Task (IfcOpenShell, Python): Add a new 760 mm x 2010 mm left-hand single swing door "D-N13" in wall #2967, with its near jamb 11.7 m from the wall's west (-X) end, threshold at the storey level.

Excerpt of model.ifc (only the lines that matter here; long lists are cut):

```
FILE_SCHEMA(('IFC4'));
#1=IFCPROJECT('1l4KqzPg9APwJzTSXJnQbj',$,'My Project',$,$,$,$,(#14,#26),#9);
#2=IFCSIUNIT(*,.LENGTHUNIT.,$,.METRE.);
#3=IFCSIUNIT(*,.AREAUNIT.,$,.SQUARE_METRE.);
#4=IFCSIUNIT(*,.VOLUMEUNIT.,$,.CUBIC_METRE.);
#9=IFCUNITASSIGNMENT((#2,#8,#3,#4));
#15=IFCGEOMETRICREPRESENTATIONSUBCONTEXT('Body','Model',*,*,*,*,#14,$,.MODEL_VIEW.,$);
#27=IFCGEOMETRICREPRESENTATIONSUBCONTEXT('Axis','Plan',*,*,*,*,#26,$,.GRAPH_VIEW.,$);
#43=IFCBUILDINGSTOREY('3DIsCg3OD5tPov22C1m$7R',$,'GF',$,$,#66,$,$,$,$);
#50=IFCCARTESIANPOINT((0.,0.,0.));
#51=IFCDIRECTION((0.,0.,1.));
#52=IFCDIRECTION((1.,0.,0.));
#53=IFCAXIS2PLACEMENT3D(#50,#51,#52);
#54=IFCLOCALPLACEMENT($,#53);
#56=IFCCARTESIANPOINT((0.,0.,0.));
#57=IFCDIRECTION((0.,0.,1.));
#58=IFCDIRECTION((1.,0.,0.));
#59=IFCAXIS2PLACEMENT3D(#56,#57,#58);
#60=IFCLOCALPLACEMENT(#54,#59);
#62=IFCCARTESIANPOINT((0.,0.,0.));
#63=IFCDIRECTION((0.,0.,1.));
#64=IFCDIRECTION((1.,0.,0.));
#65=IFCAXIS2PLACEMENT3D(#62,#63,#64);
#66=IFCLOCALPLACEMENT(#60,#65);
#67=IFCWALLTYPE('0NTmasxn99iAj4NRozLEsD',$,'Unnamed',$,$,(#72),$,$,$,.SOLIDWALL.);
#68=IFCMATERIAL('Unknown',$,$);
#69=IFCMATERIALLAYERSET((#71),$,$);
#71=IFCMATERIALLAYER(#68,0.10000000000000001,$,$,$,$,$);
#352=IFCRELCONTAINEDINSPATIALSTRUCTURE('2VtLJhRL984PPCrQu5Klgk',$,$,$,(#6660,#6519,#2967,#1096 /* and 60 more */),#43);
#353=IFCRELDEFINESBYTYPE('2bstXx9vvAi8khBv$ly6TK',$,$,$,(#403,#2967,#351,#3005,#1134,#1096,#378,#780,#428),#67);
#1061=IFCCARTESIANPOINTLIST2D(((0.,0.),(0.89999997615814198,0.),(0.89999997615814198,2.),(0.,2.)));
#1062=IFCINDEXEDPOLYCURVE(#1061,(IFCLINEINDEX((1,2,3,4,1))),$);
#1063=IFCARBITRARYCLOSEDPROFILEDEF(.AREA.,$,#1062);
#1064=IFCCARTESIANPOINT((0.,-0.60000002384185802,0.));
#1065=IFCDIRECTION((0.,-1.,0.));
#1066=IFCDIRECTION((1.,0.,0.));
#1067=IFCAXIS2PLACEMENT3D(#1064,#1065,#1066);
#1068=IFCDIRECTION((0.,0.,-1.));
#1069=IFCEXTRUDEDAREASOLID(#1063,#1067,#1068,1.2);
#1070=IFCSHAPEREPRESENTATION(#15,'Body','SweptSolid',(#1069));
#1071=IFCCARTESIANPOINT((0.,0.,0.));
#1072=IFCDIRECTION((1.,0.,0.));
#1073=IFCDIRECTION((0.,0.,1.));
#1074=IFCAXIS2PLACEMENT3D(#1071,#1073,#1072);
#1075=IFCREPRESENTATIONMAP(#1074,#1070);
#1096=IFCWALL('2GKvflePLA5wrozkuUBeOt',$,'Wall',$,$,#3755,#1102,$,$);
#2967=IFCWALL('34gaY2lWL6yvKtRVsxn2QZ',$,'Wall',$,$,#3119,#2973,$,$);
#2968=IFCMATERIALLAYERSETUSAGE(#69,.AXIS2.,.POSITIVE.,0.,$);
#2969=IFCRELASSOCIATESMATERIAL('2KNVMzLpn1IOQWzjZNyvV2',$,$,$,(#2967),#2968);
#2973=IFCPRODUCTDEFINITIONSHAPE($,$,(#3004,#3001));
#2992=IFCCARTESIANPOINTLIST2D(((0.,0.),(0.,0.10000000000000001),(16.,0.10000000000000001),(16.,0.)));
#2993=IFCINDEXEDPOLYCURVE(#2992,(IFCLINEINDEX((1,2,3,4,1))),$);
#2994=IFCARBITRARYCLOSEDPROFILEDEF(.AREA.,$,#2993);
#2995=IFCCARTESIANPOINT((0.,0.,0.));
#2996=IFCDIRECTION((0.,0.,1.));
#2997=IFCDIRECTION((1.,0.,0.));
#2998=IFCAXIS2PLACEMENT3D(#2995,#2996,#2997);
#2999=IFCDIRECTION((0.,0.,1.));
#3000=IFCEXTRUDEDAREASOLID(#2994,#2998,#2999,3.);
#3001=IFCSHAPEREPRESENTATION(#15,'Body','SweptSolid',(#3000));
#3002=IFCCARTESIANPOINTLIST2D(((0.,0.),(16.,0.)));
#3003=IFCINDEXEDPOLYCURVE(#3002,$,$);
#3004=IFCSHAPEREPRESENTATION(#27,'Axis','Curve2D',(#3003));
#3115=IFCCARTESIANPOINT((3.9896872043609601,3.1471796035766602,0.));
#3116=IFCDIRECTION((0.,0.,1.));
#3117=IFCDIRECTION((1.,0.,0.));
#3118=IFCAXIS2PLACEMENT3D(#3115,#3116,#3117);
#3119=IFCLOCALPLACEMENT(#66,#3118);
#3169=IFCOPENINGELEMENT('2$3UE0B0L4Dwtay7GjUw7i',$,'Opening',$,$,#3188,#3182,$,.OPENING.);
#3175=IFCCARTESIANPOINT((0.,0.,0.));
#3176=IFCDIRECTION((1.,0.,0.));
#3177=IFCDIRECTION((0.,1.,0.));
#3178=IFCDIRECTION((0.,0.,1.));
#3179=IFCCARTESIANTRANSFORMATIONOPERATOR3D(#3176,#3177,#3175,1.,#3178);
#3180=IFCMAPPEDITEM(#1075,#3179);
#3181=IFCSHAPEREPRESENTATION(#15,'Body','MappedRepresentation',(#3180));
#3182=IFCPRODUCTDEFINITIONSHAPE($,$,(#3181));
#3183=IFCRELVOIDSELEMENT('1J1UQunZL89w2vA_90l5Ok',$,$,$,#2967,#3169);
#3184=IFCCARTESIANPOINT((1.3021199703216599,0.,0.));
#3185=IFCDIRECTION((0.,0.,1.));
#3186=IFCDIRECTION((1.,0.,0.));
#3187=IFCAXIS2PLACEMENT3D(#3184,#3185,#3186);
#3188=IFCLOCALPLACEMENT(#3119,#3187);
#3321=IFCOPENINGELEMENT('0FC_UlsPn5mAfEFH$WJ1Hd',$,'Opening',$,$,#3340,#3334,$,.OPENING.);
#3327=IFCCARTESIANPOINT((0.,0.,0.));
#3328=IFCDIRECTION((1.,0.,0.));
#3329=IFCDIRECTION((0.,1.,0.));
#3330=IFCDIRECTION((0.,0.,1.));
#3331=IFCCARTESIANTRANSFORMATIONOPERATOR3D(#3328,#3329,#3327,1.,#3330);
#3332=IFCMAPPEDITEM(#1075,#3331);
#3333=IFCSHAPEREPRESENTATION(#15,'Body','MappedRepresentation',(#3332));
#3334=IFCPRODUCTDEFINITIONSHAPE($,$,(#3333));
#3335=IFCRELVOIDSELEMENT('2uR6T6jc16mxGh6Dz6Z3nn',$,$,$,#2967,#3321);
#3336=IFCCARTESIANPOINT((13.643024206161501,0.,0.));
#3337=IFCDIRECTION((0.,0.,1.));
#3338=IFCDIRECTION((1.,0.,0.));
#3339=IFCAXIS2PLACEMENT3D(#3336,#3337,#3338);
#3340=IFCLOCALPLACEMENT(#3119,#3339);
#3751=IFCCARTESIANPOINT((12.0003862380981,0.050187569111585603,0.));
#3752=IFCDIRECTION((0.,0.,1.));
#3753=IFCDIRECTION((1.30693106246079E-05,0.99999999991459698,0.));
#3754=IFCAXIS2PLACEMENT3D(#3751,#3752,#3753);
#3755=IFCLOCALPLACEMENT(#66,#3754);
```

```python
import numpy as np
import ifcopenshell
import ifcopenshell.api.feature
import ifcopenshell.api.geometry
import ifcopenshell.api.root
import ifcopenshell.api.spatial
import ifcopenshell.geom
import ifcopenshell.util.element
import ifcopenshell.util.placement
import ifcopenshell.util.representation
import ifcopenshell.util.shape
import ifcopenshell.util.unit

model = ifcopenshell.open("model.ifc")
unit_scale = ifcopenshell.util.unit.calculate_unit_scale(model)
settings = ifcopenshell.geom.settings()


def volume(element):
    """Net volume in cubic metres, openings subtracted."""
    shape = ifcopenshell.geom.create_shape(settings, element)
    return ifcopenshell.util.shape.get_volume(shape.geometry)


wall = model.by_id(2967)
storey = ifcopenshell.util.element.get_container(wall, ifc_class="IfcBuildingStorey")
context = ifcopenshell.util.representation.get_context(model, "Model", "Body", "MODEL_VIEW")
before = volume(wall)

width, height, from_end, sill = 0.76, 2.01, 11.7, 0.0  # metres

# The wall runs along its own X axis, and the end named is its -X end.
wall_shape = ifcopenshell.geom.create_shape(settings, wall)
x, y, z = ifcopenshell.util.shape.get_vertices(wall_shape.geometry).T
start = x.min() + from_end
face, thickness = float(y.min()), float(y.max() - y.min())
wall_matrix = ifcopenshell.util.placement.get_local_placement(wall.ObjectPlacement)
level = ifcopenshell.util.placement.get_local_placement(storey.ObjectPlacement)[2, 3]


def in_wall(x, y):
    """Placement at x, y metres in the wall's axes, at sill height."""
    matrix = wall_matrix.copy()
    matrix[:, 3] = wall_matrix @ np.array([x / unit_scale, y / unit_scale, 0.0, 1.0])
    matrix[2, 3] = level + sill / unit_scale
    return matrix


# Opening: a box that overshoots both wall faces by 50 mm.
opening = ifcopenshell.api.root.create_entity(model, ifc_class="IfcOpeningElement", predefined_type="OPENING")
box = ifcopenshell.api.geometry.add_wall_representation(
    model, context=context, length=width, height=height, thickness=thickness + 0.1
)
ifcopenshell.api.geometry.assign_representation(model, product=opening, representation=box)
ifcopenshell.api.geometry.edit_object_placement(model, product=opening, matrix=in_wall(start, face - 0.05), is_si=False)
ifcopenshell.api.feature.add_feature(model, feature=opening, element=wall)

door = ifcopenshell.api.root.create_entity(model, ifc_class="IfcDoor", name="D-N13", predefined_type="DOOR")
door.OverallWidth, door.OverallHeight = width / unit_scale, height / unit_scale
door.OperationType = "SINGLE_SWING_LEFT"
body = ifcopenshell.api.geometry.add_door_representation(
    model,
    context=context,
    overall_width=door.OverallWidth,
    overall_height=door.OverallHeight,
    operation_type="SINGLE_SWING_LEFT",
    lining_properties={"LiningDepth": thickness / unit_scale, "ThresholdDepth": thickness / unit_scale},
)
ifcopenshell.api.geometry.assign_representation(model, product=door, representation=body)
ifcopenshell.api.spatial.assign_container(model, products=[door], relating_structure=storey)
ifcopenshell.api.feature.add_filling(model, opening=opening, element=door)

# The lining spans the wall, so the door starts at the wall face.
ifcopenshell.api.geometry.edit_object_placement(model, product=door, matrix=in_wall(start, face), is_si=False)

after = volume(wall)

print(f"wall volume {before:.3f} -> {after:.3f} m3")

model.write("model_v2.ifc")
```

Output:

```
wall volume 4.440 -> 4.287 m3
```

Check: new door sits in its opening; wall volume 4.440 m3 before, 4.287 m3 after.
